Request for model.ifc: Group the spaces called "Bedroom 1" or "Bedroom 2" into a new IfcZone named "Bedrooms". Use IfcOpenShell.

First a look at what the model holds.

```python
import ifcopenshell

model = ifcopenshell.open("model.ifc")
print(model.schema)
seen = {}
for space in model.by_type("IfcSpace"):
    seen[space.LongName] = seen.get(space.LongName, 0) + 1
for name, count in sorted(seen.items(), key=str):
    print(count, "x", name)
print("zones:", [z.Name for z in model.by_type("IfcZone")][:20])
```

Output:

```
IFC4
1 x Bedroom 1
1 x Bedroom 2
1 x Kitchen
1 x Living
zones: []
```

```python
import ifcopenshell
import ifcopenshell.api.group
import ifcopenshell.api.root

model = ifcopenshell.open("model.ifc")

names = {"Bedroom 1", "Bedroom 2"}
spaces = [s for s in model.by_type("IfcSpace") if s.LongName in names]

zone = ifcopenshell.api.root.create_entity(model, ifc_class="IfcZone", name="Bedrooms")
ifcopenshell.api.group.assign_group(model, products=spaces, group=zone)
print(len(spaces), "spaces in", zone.Name)

model.write("model-out.ifc")
```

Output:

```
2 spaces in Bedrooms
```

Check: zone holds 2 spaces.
